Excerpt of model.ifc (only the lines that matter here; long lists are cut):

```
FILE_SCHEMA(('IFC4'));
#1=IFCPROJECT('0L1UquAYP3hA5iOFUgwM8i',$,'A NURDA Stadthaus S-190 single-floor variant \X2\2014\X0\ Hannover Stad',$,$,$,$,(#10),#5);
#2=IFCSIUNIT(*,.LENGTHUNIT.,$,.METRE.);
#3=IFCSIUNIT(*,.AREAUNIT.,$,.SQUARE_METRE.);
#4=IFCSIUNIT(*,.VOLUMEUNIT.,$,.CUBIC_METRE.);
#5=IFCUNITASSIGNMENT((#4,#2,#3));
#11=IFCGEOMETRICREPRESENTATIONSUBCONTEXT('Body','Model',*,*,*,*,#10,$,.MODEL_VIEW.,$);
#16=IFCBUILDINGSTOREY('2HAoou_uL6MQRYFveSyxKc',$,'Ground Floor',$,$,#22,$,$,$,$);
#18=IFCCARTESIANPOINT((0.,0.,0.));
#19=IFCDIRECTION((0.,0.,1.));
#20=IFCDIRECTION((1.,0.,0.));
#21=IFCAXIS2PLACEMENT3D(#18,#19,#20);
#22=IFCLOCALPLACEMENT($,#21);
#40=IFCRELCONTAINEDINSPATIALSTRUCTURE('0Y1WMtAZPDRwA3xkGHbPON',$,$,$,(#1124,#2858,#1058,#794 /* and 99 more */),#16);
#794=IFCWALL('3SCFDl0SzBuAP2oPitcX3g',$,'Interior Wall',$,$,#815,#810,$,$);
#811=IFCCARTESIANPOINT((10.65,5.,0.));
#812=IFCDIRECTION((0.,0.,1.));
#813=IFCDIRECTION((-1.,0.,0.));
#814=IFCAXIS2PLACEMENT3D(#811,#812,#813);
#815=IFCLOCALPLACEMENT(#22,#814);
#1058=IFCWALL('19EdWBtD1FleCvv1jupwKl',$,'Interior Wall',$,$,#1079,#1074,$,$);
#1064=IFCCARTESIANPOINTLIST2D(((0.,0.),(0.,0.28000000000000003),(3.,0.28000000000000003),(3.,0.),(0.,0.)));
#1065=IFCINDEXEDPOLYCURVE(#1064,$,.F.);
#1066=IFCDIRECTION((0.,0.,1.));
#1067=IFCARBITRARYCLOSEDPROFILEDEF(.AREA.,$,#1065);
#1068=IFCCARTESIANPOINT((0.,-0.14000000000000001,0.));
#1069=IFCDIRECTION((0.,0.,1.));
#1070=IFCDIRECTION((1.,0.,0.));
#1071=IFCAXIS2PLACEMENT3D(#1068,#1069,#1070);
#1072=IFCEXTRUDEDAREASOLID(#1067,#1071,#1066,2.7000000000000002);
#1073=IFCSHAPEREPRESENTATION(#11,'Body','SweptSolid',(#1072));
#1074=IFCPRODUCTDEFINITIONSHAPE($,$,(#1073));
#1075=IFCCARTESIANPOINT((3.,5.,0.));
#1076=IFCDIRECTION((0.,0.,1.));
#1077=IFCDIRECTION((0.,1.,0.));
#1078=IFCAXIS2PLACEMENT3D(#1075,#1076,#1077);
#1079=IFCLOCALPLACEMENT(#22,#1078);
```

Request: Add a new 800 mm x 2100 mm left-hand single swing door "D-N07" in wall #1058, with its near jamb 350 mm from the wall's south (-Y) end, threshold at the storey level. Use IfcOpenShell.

```python
import numpy as np
import ifcopenshell
import ifcopenshell.api.feature
import ifcopenshell.api.geometry
import ifcopenshell.api.root
import ifcopenshell.api.spatial
import ifcopenshell.geom
import ifcopenshell.util.element
import ifcopenshell.util.placement
import ifcopenshell.util.representation
import ifcopenshell.util.shape
import ifcopenshell.util.unit

model = ifcopenshell.open("model.ifc")
unit_scale = ifcopenshell.util.unit.calculate_unit_scale(model)
settings = ifcopenshell.geom.settings()


def volume(element):
    """Net volume in cubic metres, openings subtracted."""
    shape = ifcopenshell.geom.create_shape(settings, element)
    return ifcopenshell.util.shape.get_volume(shape.geometry)


wall = model.by_guid("19EdWBtD1FleCvv1jupwKl")
storey = ifcopenshell.util.element.get_container(wall, ifc_class="IfcBuildingStorey")
context = ifcopenshell.util.representation.get_context(model, "Model", "Body", "MODEL_VIEW")
before = volume(wall)

width, height, from_end, sill = 0.8, 2.1, 0.35, 0.0  # metres

# The wall runs along its own X axis, and the end named is its -X end.
wall_shape = ifcopenshell.geom.create_shape(settings, wall)
x, y, z = ifcopenshell.util.shape.get_vertices(wall_shape.geometry).T
start = x.min() + from_end
face, thickness = float(y.min()), float(y.max() - y.min())
wall_matrix = ifcopenshell.util.placement.get_local_placement(wall.ObjectPlacement)
level = ifcopenshell.util.placement.get_local_placement(storey.ObjectPlacement)[2, 3]


def in_wall(x, y):
    """Placement at x, y metres in the wall's axes, at sill height."""
    matrix = wall_matrix.copy()
    matrix[:, 3] = wall_matrix @ np.array([x / unit_scale, y / unit_scale, 0.0, 1.0])
    matrix[2, 3] = level + sill / unit_scale
    return matrix


# Opening: a box that overshoots both wall faces by 50 mm.
opening = ifcopenshell.api.root.create_entity(model, ifc_class="IfcOpeningElement", predefined_type="OPENING")
box = ifcopenshell.api.geometry.add_wall_representation(
    model, context=context, length=width, height=height, thickness=thickness + 0.1
)
ifcopenshell.api.geometry.assign_representation(model, product=opening, representation=box)
ifcopenshell.api.geometry.edit_object_placement(model, product=opening, matrix=in_wall(start, face - 0.05), is_si=False)
ifcopenshell.api.feature.add_feature(model, feature=opening, element=wall)

door = ifcopenshell.api.root.create_entity(model, ifc_class="IfcDoor", name="D-N07", predefined_type="DOOR")
door.OverallWidth, door.OverallHeight = width / unit_scale, height / unit_scale
door.OperationType = "SINGLE_SWING_LEFT"
body = ifcopenshell.api.geometry.add_door_representation(
    model,
    context=context,
    overall_width=door.OverallWidth,
    overall_height=door.OverallHeight,
    operation_type="SINGLE_SWING_LEFT",
    lining_properties={"LiningDepth": thickness / unit_scale, "ThresholdDepth": thickness / unit_scale},
)
ifcopenshell.api.geometry.assign_representation(model, product=door, representation=body)
ifcopenshell.api.spatial.assign_container(model, products=[door], relating_structure=storey)
ifcopenshell.api.feature.add_filling(model, opening=opening, element=door)

# The lining spans the wall, so the door starts at the wall face.
ifcopenshell.api.geometry.edit_object_placement(model, product=door, matrix=in_wall(start, face), is_si=False)

after = volume(wall)

print(f"wall volume {before:.3f} -> {after:.3f} m3")

model.write("model_updated.ifc")
```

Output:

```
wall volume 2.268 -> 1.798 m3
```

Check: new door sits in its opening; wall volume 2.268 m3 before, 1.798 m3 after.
